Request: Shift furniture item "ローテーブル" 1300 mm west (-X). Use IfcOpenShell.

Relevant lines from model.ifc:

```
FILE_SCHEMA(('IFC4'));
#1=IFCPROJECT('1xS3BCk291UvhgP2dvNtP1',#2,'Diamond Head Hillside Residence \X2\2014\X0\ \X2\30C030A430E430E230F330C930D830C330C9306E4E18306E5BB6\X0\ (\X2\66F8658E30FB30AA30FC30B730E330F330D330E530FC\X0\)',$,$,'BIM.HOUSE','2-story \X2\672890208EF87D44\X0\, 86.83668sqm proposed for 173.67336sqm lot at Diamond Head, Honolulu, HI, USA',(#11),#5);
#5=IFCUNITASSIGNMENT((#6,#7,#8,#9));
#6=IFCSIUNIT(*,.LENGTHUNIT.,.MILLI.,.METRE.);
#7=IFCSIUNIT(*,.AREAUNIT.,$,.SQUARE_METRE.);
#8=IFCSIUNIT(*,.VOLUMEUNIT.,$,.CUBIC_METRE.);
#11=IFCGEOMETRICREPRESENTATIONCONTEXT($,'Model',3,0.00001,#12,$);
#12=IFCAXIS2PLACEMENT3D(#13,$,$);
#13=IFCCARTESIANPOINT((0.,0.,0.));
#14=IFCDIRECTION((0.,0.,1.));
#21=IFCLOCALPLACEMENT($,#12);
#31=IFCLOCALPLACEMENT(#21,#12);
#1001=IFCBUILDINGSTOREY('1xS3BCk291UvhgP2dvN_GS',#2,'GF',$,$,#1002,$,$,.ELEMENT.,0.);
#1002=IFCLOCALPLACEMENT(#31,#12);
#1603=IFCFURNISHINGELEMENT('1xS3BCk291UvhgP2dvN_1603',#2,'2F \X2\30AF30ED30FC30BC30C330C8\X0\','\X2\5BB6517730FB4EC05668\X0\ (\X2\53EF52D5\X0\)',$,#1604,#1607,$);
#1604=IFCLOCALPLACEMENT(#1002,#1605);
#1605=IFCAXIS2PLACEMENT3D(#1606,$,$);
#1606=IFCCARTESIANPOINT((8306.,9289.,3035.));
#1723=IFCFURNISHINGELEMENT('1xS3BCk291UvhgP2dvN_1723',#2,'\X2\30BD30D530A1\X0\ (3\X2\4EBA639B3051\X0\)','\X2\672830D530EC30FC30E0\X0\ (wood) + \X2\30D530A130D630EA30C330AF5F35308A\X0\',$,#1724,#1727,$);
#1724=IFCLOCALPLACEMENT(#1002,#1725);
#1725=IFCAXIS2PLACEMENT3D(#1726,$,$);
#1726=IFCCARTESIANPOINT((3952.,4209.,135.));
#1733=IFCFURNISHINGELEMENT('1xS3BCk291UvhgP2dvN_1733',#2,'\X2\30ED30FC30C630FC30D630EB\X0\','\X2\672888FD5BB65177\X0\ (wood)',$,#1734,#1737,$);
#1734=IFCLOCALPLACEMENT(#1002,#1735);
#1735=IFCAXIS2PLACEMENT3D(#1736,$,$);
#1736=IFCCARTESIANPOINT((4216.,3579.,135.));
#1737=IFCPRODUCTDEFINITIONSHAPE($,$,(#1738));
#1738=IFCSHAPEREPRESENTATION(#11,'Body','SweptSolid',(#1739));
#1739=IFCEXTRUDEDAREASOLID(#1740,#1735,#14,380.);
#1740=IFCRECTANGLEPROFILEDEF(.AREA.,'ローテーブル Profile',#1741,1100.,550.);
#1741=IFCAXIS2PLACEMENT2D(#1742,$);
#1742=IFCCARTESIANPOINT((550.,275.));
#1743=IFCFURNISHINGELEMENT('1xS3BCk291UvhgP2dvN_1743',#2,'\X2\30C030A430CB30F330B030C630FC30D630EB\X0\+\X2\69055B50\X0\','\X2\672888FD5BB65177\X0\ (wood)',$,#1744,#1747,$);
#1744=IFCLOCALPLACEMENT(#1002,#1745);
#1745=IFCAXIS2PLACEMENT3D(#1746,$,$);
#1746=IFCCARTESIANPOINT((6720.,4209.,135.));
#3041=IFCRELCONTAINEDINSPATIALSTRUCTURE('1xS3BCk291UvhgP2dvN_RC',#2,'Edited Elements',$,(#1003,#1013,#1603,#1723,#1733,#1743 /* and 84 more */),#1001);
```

```python
import ifcopenshell
import ifcopenshell.api.geometry
import ifcopenshell.util.placement
import ifcopenshell.util.unit

model = ifcopenshell.open("model.ifc")
unit_scale = ifcopenshell.util.unit.calculate_unit_scale(model)

item = model.by_guid("1xS3BCk291UvhgP2dvN_1733")
matrix = ifcopenshell.util.placement.get_local_placement(item.ObjectPlacement)
matrix[0, 3] -= 1.3 / unit_scale
ifcopenshell.api.geometry.edit_object_placement(model, product=item, matrix=matrix, is_si=False)

print(ifcopenshell.util.placement.get_local_placement(item.ObjectPlacement).round(3) + 0.0)

model.write("model_updated.ifc")
```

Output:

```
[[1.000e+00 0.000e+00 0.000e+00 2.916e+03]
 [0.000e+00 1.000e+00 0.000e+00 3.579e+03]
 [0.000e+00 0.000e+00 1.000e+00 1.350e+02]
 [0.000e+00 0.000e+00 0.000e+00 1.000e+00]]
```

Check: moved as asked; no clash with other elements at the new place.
